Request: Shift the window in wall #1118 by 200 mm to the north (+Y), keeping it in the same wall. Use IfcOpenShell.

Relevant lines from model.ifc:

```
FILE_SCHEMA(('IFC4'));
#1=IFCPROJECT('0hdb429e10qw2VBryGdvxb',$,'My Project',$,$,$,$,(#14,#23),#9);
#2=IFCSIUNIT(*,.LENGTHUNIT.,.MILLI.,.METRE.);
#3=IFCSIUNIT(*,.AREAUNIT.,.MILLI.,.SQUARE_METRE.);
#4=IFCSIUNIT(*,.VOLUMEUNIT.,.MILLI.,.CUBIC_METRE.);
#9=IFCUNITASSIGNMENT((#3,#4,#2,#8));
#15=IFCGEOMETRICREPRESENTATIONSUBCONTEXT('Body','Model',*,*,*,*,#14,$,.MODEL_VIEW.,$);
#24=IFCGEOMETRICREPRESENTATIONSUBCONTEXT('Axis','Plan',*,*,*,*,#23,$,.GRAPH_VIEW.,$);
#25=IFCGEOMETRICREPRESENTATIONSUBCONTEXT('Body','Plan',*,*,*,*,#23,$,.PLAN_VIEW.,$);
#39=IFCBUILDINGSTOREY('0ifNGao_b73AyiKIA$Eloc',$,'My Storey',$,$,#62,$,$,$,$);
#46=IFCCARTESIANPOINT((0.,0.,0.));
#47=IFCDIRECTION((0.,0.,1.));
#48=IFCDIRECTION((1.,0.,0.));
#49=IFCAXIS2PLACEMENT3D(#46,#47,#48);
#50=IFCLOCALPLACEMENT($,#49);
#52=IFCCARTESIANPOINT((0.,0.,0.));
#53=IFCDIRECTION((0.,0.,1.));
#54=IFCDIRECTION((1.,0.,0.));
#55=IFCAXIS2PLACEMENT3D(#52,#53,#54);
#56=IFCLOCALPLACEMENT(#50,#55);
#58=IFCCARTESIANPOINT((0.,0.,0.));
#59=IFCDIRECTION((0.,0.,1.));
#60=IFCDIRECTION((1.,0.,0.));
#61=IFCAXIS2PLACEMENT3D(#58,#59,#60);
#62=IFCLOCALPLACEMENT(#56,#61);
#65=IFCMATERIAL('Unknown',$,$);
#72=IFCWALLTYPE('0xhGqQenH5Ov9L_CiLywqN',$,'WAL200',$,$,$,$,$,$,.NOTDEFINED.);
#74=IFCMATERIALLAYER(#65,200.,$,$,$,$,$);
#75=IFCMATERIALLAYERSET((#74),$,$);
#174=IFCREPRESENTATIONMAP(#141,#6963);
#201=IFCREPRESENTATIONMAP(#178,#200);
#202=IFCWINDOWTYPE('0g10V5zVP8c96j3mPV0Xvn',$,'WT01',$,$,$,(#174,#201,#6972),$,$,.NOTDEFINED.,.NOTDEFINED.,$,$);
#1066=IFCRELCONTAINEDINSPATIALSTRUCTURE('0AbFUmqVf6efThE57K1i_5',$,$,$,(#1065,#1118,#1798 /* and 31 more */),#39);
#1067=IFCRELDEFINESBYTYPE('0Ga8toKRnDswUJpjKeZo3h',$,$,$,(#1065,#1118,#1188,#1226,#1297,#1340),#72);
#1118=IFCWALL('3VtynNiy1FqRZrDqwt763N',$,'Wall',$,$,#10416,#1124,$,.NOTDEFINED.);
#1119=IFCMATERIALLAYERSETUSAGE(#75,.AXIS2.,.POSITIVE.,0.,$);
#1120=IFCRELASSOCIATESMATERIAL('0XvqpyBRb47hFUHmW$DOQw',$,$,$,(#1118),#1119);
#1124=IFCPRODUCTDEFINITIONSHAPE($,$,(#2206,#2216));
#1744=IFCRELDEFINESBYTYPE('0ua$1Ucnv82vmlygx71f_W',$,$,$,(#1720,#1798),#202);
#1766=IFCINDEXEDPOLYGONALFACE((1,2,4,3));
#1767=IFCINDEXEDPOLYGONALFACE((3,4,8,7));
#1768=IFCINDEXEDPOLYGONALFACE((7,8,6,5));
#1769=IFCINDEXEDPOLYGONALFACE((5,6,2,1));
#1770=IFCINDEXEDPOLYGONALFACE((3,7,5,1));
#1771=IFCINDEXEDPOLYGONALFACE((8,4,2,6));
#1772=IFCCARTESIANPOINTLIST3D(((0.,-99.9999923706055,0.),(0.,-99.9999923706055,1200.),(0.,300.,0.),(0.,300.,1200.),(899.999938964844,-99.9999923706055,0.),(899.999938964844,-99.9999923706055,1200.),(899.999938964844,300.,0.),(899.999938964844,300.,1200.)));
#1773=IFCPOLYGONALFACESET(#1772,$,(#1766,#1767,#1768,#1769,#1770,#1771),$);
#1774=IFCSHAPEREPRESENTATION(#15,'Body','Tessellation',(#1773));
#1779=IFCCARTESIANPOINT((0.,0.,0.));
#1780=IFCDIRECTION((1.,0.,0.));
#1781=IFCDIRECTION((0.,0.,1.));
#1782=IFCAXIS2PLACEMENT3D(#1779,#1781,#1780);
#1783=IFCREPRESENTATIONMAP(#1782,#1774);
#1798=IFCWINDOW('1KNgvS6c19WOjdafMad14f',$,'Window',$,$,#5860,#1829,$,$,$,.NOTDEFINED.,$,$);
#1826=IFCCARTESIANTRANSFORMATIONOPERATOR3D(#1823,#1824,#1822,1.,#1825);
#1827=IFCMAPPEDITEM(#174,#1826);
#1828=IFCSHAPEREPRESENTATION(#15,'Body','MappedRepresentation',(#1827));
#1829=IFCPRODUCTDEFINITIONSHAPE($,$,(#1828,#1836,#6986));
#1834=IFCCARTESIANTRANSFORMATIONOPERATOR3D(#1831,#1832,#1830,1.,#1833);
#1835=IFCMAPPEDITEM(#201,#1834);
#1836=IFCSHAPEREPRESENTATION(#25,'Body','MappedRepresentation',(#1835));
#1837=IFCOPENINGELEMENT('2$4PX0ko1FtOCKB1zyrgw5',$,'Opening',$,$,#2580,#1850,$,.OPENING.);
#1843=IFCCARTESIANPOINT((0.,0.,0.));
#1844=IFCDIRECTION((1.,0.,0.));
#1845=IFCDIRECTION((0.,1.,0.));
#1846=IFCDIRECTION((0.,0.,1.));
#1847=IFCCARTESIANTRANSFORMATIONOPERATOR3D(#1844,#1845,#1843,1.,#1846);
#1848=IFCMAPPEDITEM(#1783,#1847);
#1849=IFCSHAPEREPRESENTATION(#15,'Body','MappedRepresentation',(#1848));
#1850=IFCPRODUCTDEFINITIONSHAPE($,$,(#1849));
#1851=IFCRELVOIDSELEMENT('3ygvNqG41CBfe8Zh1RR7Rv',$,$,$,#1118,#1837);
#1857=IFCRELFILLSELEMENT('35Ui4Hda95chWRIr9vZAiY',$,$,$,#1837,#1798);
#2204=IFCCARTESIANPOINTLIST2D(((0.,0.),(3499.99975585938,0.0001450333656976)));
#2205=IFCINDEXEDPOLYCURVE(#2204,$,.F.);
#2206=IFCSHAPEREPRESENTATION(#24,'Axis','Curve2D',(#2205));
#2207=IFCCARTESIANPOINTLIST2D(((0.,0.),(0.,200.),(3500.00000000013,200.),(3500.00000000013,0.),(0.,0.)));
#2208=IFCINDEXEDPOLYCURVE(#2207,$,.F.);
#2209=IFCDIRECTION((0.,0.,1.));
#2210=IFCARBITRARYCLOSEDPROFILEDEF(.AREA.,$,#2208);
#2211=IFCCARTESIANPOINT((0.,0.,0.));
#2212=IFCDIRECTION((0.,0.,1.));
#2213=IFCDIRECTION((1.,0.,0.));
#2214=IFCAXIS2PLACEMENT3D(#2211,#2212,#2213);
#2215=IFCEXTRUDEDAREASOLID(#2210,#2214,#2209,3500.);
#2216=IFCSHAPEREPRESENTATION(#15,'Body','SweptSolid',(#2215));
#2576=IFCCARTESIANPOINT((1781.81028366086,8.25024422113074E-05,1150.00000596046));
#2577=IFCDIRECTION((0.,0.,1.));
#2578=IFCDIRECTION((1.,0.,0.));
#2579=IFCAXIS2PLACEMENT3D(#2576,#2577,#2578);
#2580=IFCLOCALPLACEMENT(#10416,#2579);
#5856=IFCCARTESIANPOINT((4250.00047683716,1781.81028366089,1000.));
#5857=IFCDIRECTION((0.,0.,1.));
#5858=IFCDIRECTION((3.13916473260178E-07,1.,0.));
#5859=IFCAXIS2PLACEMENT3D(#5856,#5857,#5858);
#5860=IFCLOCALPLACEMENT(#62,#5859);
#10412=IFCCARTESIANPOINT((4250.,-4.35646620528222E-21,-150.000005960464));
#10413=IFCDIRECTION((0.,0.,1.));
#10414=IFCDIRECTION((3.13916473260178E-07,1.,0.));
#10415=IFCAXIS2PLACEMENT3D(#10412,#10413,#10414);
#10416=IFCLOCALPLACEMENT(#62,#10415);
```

```python
import ifcopenshell
import ifcopenshell.api.geometry
import ifcopenshell.util.placement
import ifcopenshell.util.unit

model = ifcopenshell.open("model.ifc")
unit_scale = ifcopenshell.util.unit.calculate_unit_scale(model)

window = model.by_id(1798)
opening = window.FillsVoids[0].RelatingOpeningElement
wall = opening.VoidsElements[0].RelatingBuildingElement

wall_matrix = ifcopenshell.util.placement.get_local_placement(wall.ObjectPlacement)
shift = wall_matrix[:3, 0] * 0.2 / unit_scale
before = ifcopenshell.util.placement.get_local_placement(window.ObjectPlacement)[:3, 3].copy()

# The window is not placed relative to its opening, so move both.
for product in (opening, window):
    matrix = ifcopenshell.util.placement.get_local_placement(product.ObjectPlacement)
    matrix[:3, 3] += shift
    ifcopenshell.api.geometry.edit_object_placement(model, product=product, matrix=matrix, is_si=False)

after = ifcopenshell.util.placement.get_local_placement(window.ObjectPlacement)[:3, 3]
print("window moved by", (after - before).round(3) + 0.0)

model.write("model_v2.ifc")
```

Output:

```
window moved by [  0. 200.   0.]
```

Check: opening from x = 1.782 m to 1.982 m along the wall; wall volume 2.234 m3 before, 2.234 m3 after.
